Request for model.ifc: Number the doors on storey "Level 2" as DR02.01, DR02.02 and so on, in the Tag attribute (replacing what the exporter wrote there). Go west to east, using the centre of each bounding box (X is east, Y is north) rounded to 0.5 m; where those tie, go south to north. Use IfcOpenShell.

First a look at what the model holds.

```python
import ifcopenshell
import ifcopenshell.util.element
import ifcopenshell.util.placement

model = ifcopenshell.open("model.ifc")
print(model.schema)
storey = next(s for s in model.by_type("IfcBuildingStorey") if s.Name == "Level 2")
doors = [e for e in ifcopenshell.util.element.get_decomposition(storey) if e.is_a("IfcDoor")]
for e in sorted(doors, key=lambda e: e.id()):
    origin = ifcopenshell.util.placement.get_local_placement(e.ObjectPlacement)[:3, 3]
    print(e.id(), e.Tag, e.Name, origin.round(2) + 0.0, sep=" | ")
```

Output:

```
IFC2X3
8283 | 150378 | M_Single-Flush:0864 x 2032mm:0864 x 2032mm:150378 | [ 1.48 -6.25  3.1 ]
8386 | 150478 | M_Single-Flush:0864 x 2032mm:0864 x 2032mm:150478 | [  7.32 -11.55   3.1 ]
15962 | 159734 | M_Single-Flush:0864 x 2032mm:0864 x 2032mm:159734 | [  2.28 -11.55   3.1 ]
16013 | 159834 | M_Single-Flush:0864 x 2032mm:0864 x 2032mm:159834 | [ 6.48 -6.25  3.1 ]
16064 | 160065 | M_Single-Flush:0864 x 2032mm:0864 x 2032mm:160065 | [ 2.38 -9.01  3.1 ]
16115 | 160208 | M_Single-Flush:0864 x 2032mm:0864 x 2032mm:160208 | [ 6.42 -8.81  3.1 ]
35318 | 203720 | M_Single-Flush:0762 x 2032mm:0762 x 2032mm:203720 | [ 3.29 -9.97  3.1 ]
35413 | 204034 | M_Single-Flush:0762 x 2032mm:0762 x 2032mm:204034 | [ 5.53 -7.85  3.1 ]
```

```python
import ifcopenshell
import ifcopenshell.geom
import ifcopenshell.util.element
import ifcopenshell.util.shape

model = ifcopenshell.open("model.ifc")
settings = ifcopenshell.geom.settings()
settings.set("use-world-coords", True)


def centre(element):
    shape = ifcopenshell.geom.create_shape(settings, element)
    return ifcopenshell.util.shape.get_bbox_centroid(shape.geometry)


storey = next(s for s in model.by_type("IfcBuildingStorey") if s.Name == "Level 2")
doors = [e for e in ifcopenshell.util.element.get_decomposition(storey) if e.is_a("IfcDoor")]

# Insertion points can sit at a corner or the storey origin, so sort by the geometry (in metres).
centres = {e: centre(e) for e in doors}
doors.sort(key=lambda e: (round(centres[e][0] / 0.5), centres[e][1]))

for i, e in enumerate(doors, start=1):
    number = f"DR02.{i:02d}"
    e.Tag = number
    print(e.id(), number)

model.write("model_rev.ifc")
```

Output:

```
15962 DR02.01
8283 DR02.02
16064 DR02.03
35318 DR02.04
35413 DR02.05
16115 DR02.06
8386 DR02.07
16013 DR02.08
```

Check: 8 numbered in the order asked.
